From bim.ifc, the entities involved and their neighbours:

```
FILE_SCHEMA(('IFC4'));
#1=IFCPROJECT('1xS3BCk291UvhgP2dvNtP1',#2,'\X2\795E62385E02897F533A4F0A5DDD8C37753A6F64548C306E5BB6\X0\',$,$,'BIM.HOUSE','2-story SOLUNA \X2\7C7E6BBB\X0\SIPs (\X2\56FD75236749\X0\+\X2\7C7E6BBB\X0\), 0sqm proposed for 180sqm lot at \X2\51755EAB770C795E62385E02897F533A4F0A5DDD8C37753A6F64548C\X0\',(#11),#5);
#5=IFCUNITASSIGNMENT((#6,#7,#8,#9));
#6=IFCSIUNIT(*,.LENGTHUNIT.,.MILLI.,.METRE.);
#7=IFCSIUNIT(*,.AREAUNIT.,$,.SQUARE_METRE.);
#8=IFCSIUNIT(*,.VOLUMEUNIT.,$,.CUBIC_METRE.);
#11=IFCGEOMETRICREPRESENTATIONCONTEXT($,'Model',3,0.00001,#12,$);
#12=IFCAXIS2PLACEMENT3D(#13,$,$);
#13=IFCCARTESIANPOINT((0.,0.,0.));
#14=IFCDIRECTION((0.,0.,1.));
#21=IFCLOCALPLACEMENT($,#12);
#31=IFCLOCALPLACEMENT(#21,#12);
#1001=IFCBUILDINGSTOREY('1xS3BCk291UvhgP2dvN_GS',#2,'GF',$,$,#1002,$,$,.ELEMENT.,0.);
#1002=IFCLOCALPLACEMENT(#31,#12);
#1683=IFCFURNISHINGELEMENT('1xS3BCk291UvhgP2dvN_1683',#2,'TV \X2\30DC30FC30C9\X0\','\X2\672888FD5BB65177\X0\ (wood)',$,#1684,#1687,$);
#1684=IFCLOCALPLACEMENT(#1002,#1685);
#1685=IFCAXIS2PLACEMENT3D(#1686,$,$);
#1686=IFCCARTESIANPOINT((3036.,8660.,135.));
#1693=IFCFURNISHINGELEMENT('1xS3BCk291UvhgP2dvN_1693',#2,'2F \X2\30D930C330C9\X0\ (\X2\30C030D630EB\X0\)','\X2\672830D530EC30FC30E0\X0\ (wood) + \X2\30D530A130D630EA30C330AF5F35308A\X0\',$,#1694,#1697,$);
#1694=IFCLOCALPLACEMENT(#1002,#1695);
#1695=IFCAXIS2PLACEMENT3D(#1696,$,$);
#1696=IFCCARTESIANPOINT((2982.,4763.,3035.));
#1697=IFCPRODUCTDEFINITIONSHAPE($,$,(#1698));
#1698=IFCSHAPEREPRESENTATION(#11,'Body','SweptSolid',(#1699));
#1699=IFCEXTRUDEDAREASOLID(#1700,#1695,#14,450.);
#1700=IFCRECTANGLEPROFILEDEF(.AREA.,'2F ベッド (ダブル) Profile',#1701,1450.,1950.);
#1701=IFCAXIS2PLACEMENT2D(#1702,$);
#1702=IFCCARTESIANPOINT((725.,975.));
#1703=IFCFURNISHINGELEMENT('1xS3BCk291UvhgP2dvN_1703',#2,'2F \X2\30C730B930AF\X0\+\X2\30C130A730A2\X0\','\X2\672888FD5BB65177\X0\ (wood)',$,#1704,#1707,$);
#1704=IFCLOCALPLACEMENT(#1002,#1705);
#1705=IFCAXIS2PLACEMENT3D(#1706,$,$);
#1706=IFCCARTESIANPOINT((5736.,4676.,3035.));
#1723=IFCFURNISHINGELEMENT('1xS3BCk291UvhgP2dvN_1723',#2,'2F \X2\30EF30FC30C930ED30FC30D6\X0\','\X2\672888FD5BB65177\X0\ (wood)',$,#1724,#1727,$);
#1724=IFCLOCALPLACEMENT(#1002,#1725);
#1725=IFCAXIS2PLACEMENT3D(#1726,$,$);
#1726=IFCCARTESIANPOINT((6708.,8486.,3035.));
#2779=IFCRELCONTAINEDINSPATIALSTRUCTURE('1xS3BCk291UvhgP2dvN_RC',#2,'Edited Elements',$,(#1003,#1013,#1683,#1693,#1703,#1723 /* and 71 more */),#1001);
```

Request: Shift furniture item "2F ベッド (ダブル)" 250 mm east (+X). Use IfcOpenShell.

```python
import ifcopenshell
import ifcopenshell.api.geometry
import ifcopenshell.util.placement
import ifcopenshell.util.unit

model = ifcopenshell.open("bim.ifc")
unit_scale = ifcopenshell.util.unit.calculate_unit_scale(model)

item = model.by_guid("1xS3BCk291UvhgP2dvN_1693")
matrix = ifcopenshell.util.placement.get_local_placement(item.ObjectPlacement)
matrix[0, 3] += 0.25 / unit_scale
ifcopenshell.api.geometry.edit_object_placement(model, product=item, matrix=matrix, is_si=False)

print(ifcopenshell.util.placement.get_local_placement(item.ObjectPlacement).round(3) + 0.0)

model.write("bim_rev.ifc")
```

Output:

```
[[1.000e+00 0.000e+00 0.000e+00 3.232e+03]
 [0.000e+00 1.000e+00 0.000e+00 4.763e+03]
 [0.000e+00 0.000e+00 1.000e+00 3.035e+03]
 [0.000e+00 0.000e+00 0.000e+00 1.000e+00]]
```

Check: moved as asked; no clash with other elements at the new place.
